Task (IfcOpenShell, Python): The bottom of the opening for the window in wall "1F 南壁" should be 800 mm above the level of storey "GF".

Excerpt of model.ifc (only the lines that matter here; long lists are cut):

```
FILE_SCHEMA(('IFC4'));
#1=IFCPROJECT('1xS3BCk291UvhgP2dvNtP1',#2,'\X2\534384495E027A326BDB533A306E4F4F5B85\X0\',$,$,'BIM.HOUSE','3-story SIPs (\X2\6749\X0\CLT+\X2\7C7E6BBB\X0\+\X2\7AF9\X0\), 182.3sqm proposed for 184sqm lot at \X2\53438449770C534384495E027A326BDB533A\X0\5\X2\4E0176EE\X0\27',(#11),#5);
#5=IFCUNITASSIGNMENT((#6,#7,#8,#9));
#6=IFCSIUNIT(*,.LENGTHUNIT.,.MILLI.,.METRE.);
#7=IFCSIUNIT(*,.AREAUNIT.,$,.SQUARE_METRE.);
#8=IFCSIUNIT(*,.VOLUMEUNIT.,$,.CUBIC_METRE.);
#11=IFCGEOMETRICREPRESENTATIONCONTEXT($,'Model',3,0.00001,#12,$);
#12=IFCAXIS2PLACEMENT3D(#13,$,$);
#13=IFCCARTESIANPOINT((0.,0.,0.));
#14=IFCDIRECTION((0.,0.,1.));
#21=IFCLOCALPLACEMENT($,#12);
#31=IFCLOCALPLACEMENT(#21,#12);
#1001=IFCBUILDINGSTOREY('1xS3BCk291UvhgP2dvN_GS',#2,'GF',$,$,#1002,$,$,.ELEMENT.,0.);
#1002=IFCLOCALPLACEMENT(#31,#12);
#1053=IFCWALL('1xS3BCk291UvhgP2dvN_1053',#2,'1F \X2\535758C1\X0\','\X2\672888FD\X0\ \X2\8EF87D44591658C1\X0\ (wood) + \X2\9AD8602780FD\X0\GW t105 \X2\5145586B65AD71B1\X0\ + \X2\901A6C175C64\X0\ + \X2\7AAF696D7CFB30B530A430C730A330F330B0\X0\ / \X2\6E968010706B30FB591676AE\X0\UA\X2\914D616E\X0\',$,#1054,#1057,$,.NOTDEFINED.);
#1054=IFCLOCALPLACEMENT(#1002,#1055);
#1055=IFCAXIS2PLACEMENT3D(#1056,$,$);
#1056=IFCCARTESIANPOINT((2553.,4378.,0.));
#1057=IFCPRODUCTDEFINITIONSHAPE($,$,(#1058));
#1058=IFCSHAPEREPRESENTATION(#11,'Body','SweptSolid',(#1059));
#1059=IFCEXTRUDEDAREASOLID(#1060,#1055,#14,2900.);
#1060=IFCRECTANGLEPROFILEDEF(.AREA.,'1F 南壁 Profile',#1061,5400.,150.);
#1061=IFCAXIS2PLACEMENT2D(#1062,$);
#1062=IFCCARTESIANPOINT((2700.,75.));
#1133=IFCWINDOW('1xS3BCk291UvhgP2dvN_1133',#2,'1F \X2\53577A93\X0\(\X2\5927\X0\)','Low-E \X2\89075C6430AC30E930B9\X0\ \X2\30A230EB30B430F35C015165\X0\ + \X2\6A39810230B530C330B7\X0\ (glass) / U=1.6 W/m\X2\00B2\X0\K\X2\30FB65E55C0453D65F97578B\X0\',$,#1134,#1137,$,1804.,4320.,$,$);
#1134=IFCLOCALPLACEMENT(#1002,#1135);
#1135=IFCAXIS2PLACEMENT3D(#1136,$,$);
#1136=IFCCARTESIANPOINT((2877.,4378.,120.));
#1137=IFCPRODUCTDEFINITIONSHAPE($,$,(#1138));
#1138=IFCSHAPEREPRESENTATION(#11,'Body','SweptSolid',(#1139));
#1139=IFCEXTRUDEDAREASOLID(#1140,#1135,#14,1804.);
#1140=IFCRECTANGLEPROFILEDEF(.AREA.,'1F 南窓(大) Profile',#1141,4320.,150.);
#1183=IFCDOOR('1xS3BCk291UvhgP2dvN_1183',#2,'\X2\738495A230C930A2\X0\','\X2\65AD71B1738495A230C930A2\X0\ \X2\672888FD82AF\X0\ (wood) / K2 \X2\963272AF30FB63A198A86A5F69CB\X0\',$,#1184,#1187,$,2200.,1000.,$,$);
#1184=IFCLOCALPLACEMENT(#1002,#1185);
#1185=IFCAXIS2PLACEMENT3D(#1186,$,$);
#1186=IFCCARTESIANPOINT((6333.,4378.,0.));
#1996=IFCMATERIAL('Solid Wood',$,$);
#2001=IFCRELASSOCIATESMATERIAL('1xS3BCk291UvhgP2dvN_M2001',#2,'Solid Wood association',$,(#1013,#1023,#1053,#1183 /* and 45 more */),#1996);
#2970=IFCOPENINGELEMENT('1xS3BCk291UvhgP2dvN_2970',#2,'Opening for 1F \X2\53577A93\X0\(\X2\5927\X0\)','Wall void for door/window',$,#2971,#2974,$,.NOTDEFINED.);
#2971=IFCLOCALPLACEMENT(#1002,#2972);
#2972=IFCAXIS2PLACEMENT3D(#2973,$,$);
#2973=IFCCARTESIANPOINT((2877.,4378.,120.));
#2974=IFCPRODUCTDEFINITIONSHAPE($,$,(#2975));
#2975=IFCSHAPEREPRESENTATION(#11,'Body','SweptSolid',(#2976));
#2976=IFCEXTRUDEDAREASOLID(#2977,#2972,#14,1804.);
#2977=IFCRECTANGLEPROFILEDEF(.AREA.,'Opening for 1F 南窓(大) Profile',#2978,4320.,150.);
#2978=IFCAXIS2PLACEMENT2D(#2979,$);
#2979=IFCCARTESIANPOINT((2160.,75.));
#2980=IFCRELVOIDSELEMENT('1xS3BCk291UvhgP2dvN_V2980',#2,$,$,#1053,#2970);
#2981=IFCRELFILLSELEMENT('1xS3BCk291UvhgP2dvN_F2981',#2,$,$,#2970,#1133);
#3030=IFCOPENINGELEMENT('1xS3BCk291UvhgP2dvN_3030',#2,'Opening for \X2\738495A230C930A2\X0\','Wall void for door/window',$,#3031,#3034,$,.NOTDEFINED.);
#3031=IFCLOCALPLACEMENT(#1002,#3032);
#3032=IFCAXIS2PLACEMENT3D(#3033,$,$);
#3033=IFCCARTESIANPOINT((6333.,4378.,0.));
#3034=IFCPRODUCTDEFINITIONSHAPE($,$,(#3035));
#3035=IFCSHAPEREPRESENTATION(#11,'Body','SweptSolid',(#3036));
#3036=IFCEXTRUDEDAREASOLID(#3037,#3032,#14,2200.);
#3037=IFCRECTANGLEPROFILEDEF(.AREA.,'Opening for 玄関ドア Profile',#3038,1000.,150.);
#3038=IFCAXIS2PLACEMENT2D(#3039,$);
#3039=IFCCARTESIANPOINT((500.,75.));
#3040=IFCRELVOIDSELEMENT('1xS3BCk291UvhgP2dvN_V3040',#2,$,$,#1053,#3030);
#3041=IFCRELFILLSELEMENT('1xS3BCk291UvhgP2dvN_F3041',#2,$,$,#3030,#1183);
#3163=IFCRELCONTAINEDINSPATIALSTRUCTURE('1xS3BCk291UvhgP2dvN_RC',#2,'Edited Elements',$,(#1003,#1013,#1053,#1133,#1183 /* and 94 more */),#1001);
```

```python
import numpy as np
import ifcopenshell
import ifcopenshell.api.geometry
import ifcopenshell.geom
import ifcopenshell.util.element
import ifcopenshell.util.placement
import ifcopenshell.util.shape
import ifcopenshell.util.unit

model = ifcopenshell.open("model.ifc")
unit_scale = ifcopenshell.util.unit.calculate_unit_scale(model)

window = model.by_id(1133)
opening = window.FillsVoids[0].RelatingOpeningElement
storey = ifcopenshell.util.element.get_container(window, ifc_class="IfcBuildingStorey")
level = ifcopenshell.util.placement.get_local_placement(storey.ObjectPlacement)[2, 3]

# The opening's origin need not be at the sill, so measure its lowest point.
shape = ifcopenshell.geom.create_shape(ifcopenshell.geom.settings(), opening)
bottom = ifcopenshell.util.shape.get_shape_bottom_elevation(shape, shape.geometry) / unit_scale
dz = level + 800.0 - bottom

shift = np.array([0.0, 0.0, dz])
# The window is not placed relative to its opening, so move both.
for product in (opening, window):
    matrix = ifcopenshell.util.placement.get_local_placement(product.ObjectPlacement)
    matrix[:3, 3] += shift
    ifcopenshell.api.geometry.edit_object_placement(model, product=product, matrix=matrix, is_si=False)

print(f"moved by {dz * unit_scale:+.3f} m")

model.write("model-out.ifc")
```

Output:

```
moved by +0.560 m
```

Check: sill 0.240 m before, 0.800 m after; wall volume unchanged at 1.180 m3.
